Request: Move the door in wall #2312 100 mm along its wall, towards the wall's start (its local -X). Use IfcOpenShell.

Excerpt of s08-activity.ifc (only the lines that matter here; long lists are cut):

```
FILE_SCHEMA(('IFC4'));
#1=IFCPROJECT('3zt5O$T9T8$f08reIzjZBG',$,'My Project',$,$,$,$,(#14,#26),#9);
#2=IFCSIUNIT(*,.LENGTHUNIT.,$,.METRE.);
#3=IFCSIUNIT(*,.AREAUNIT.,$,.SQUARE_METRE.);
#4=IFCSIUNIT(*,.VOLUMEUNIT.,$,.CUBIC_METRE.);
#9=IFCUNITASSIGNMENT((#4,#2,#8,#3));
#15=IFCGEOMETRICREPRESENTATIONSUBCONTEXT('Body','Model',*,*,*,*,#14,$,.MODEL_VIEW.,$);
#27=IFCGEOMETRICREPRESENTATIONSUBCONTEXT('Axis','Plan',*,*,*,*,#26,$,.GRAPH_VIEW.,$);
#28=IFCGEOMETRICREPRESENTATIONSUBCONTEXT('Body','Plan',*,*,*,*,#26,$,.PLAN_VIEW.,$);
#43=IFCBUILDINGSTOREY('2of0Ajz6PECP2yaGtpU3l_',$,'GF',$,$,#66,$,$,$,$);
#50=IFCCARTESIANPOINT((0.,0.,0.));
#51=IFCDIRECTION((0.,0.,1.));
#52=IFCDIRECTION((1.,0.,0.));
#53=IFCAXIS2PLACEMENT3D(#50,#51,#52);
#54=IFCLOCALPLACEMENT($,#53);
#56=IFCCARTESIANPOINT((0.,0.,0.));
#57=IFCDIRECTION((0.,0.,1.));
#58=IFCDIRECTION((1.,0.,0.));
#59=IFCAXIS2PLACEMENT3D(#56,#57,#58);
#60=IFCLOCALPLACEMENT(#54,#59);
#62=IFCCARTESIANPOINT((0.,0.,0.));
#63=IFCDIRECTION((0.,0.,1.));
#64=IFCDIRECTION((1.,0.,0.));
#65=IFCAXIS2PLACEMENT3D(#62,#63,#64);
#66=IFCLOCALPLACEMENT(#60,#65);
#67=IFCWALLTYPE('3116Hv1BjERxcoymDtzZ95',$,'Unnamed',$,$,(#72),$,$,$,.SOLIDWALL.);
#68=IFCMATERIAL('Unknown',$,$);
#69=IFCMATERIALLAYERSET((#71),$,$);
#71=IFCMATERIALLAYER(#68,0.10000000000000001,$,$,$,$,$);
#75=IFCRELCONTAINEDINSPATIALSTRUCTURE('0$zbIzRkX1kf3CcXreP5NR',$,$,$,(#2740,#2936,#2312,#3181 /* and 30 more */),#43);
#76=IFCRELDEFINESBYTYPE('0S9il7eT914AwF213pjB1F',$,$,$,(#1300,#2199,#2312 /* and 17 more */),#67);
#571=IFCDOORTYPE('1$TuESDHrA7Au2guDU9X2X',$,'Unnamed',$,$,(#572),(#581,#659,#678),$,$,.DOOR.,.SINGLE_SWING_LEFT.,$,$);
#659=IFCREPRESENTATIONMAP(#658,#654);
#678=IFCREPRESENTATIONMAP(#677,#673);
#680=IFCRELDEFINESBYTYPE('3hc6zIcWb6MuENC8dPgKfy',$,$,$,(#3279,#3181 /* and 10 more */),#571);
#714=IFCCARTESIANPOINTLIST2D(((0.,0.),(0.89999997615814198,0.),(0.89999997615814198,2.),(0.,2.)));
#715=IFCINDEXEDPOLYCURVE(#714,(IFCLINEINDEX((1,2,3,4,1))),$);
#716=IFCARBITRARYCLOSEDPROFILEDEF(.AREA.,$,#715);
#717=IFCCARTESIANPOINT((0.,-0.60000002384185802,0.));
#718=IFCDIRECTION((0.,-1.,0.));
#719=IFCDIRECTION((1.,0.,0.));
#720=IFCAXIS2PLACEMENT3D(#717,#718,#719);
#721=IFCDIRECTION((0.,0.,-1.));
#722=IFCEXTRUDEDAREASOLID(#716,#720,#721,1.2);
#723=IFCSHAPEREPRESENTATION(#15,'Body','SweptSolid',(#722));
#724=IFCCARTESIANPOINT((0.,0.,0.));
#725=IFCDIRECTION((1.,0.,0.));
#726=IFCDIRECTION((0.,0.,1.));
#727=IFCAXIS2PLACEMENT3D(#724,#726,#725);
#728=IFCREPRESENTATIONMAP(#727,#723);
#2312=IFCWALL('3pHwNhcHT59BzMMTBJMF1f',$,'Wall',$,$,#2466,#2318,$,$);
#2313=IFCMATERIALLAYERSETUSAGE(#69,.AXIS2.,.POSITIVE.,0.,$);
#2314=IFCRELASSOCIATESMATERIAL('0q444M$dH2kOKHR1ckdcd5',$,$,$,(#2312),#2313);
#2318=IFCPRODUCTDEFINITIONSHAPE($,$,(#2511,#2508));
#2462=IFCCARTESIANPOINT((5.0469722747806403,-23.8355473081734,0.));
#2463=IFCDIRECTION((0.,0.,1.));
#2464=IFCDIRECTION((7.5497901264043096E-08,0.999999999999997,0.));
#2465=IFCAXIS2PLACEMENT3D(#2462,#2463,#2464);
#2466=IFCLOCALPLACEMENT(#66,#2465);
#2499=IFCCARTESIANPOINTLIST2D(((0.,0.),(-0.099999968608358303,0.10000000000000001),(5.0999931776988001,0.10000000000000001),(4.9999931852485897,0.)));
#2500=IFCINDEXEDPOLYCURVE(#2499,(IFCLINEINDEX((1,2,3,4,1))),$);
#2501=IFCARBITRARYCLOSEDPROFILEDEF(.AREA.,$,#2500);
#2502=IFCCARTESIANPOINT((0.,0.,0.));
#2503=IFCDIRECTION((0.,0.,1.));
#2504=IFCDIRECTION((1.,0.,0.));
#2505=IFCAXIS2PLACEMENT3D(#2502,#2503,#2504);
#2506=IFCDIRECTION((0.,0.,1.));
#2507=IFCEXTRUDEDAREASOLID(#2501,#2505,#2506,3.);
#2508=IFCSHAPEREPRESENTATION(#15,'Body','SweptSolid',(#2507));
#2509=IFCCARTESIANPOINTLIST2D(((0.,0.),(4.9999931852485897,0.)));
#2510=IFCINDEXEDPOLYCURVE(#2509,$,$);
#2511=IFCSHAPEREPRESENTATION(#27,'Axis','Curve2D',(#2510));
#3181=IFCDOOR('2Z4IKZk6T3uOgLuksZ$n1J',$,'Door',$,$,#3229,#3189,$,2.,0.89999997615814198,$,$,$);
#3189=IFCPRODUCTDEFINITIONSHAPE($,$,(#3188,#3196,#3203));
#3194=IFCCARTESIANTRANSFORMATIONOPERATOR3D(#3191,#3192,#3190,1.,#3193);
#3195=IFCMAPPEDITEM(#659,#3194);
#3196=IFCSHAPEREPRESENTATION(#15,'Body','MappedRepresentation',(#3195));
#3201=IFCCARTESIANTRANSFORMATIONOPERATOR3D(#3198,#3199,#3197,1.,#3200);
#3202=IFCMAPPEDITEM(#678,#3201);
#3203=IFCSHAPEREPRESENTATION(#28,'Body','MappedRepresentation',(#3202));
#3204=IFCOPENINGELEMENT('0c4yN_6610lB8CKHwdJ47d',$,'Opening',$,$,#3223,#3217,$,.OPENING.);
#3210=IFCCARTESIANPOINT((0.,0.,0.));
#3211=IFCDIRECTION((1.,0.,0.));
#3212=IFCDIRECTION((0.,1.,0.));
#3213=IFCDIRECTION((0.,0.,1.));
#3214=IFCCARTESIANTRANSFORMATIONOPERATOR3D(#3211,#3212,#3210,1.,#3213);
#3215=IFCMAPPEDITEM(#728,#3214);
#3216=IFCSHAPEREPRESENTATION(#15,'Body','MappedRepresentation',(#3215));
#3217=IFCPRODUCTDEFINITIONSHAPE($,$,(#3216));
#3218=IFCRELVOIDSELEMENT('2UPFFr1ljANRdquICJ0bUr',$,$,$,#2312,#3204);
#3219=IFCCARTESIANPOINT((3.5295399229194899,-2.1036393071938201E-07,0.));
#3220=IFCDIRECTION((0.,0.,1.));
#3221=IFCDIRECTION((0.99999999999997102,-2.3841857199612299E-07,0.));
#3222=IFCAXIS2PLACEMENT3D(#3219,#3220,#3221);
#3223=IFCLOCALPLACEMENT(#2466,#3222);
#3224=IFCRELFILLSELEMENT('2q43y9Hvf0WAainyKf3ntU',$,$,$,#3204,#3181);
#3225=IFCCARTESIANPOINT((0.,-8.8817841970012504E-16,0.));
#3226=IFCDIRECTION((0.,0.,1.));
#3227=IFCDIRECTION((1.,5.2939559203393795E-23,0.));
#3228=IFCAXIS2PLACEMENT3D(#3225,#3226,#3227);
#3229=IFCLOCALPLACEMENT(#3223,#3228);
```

```python
import ifcopenshell
import ifcopenshell.api.geometry
import ifcopenshell.util.placement
import ifcopenshell.util.unit

model = ifcopenshell.open("s08-activity.ifc")
unit_scale = ifcopenshell.util.unit.calculate_unit_scale(model)

door = model.by_guid("2Z4IKZk6T3uOgLuksZ$n1J")
opening = door.FillsVoids[0].RelatingOpeningElement
wall = opening.VoidsElements[0].RelatingBuildingElement

wall_matrix = ifcopenshell.util.placement.get_local_placement(wall.ObjectPlacement)
shift = wall_matrix[:3, 0] * -0.1 / unit_scale
before = ifcopenshell.util.placement.get_local_placement(door.ObjectPlacement)[:3, 3].copy()

# The door is placed relative to its opening, so it follows when the opening moves.
matrix = ifcopenshell.util.placement.get_local_placement(opening.ObjectPlacement)
matrix[:3, 3] += shift
ifcopenshell.api.geometry.edit_object_placement(
    model, product=opening, matrix=matrix, is_si=False, should_transform_children=True
)

after = ifcopenshell.util.placement.get_local_placement(door.ObjectPlacement)[:3, 3]
print("door moved by", (after - before).round(3) + 0.0)

model.write("s08-activity_updated.ifc")
```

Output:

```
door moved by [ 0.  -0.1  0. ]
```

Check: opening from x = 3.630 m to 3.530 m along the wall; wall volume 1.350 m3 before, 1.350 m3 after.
